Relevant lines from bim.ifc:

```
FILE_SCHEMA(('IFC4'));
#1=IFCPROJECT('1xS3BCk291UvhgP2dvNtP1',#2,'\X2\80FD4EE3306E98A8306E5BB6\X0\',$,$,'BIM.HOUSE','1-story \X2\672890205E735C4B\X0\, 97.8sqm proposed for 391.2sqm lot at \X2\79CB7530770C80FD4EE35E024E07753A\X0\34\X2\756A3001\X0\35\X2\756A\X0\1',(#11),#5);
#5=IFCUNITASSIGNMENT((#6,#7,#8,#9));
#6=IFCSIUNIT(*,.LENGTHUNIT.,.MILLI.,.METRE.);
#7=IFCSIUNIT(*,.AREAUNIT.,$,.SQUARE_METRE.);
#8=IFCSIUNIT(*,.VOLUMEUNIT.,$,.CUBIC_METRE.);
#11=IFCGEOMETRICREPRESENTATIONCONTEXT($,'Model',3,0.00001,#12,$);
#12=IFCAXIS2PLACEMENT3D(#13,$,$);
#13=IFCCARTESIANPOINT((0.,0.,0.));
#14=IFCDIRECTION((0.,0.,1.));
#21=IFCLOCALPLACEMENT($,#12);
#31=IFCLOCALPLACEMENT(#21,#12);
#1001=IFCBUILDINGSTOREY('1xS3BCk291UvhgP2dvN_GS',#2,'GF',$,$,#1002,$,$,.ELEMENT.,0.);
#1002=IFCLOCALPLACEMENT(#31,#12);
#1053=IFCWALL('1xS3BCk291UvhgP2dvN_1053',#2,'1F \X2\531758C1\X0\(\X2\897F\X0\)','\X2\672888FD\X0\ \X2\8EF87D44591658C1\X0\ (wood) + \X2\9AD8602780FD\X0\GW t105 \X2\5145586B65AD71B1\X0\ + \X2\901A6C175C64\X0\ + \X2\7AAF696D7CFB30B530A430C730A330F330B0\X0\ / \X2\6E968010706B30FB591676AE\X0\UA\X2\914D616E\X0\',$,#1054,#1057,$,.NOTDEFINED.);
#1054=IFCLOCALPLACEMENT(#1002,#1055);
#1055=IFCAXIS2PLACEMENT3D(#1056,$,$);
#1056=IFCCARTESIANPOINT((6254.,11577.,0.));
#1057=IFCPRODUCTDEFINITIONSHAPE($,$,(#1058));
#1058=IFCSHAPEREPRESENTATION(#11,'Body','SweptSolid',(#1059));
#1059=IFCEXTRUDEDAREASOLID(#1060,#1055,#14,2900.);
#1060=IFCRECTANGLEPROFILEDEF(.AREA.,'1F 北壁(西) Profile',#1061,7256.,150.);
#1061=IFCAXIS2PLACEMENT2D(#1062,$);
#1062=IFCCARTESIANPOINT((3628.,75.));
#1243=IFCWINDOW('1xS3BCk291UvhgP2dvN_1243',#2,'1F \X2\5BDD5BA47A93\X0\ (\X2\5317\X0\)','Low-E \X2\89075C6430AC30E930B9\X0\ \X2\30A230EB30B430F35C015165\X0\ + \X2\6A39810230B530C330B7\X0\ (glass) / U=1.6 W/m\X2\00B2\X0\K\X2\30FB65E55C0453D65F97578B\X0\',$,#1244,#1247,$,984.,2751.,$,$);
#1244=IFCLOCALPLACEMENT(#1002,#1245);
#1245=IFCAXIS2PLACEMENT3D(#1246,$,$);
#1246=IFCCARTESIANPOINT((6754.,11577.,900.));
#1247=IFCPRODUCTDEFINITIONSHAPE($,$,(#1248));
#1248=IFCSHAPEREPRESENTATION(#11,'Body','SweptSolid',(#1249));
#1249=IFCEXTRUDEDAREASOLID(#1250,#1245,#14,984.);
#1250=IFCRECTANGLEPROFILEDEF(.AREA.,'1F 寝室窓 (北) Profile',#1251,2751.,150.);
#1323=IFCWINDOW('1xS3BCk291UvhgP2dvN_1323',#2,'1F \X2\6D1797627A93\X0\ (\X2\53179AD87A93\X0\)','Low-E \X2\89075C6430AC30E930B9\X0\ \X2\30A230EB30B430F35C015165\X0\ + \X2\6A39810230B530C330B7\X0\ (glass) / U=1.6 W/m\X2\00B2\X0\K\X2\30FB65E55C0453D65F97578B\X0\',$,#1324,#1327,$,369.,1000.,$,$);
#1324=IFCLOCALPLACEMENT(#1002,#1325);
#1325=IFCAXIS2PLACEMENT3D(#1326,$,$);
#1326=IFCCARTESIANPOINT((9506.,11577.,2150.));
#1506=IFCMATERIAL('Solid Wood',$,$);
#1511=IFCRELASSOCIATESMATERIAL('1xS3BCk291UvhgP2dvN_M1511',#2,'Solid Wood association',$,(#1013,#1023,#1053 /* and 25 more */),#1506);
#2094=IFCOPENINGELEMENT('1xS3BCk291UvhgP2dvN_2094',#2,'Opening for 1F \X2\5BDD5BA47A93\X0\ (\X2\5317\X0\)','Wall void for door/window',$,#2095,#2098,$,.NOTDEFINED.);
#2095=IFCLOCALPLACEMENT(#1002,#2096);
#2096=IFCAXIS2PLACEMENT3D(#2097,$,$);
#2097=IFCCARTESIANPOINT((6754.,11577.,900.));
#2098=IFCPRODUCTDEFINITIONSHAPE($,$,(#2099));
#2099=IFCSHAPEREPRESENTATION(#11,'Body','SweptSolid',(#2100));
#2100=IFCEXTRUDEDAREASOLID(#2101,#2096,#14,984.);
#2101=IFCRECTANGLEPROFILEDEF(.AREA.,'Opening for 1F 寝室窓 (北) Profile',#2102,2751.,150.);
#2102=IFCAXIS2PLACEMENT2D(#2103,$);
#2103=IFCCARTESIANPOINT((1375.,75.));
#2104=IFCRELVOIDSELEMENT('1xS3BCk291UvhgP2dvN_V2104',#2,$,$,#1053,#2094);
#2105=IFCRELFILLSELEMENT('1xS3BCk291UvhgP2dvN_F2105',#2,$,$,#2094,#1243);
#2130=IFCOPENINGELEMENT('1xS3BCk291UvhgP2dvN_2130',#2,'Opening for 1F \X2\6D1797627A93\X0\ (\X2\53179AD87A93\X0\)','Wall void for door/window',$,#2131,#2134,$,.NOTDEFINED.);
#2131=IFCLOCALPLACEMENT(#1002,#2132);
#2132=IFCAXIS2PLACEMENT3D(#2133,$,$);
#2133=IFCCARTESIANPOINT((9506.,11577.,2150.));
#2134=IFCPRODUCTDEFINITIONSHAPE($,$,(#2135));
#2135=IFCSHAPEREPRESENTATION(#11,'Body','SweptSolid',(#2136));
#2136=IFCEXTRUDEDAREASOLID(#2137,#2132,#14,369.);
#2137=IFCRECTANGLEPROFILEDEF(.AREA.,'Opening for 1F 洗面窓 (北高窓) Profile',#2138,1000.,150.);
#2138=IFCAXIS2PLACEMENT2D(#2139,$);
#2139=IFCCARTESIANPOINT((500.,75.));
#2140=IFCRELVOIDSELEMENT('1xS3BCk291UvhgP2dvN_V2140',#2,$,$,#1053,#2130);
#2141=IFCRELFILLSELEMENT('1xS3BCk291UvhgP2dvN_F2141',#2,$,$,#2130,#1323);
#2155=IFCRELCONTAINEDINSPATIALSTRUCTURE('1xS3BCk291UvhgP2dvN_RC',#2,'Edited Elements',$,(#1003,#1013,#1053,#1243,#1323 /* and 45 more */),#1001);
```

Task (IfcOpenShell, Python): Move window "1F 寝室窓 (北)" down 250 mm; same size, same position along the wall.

```python
import numpy as np
import ifcopenshell
import ifcopenshell.api.geometry
import ifcopenshell.util.placement
import ifcopenshell.util.unit

model = ifcopenshell.open("bim.ifc")
unit_scale = ifcopenshell.util.unit.calculate_unit_scale(model)

window = model.by_guid("1xS3BCk291UvhgP2dvN_1243")
opening = window.FillsVoids[0].RelatingOpeningElement
dz = -0.25 / unit_scale

shift = np.array([0.0, 0.0, dz])
# The window is not placed relative to its opening, so move both.
for product in (opening, window):
    matrix = ifcopenshell.util.placement.get_local_placement(product.ObjectPlacement)
    matrix[:3, 3] += shift
    ifcopenshell.api.geometry.edit_object_placement(model, product=product, matrix=matrix, is_si=False)

print(f"moved by {dz * unit_scale:+.3f} m")

model.write("bim-out.ifc")
```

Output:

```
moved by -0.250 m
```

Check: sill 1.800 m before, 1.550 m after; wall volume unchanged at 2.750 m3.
